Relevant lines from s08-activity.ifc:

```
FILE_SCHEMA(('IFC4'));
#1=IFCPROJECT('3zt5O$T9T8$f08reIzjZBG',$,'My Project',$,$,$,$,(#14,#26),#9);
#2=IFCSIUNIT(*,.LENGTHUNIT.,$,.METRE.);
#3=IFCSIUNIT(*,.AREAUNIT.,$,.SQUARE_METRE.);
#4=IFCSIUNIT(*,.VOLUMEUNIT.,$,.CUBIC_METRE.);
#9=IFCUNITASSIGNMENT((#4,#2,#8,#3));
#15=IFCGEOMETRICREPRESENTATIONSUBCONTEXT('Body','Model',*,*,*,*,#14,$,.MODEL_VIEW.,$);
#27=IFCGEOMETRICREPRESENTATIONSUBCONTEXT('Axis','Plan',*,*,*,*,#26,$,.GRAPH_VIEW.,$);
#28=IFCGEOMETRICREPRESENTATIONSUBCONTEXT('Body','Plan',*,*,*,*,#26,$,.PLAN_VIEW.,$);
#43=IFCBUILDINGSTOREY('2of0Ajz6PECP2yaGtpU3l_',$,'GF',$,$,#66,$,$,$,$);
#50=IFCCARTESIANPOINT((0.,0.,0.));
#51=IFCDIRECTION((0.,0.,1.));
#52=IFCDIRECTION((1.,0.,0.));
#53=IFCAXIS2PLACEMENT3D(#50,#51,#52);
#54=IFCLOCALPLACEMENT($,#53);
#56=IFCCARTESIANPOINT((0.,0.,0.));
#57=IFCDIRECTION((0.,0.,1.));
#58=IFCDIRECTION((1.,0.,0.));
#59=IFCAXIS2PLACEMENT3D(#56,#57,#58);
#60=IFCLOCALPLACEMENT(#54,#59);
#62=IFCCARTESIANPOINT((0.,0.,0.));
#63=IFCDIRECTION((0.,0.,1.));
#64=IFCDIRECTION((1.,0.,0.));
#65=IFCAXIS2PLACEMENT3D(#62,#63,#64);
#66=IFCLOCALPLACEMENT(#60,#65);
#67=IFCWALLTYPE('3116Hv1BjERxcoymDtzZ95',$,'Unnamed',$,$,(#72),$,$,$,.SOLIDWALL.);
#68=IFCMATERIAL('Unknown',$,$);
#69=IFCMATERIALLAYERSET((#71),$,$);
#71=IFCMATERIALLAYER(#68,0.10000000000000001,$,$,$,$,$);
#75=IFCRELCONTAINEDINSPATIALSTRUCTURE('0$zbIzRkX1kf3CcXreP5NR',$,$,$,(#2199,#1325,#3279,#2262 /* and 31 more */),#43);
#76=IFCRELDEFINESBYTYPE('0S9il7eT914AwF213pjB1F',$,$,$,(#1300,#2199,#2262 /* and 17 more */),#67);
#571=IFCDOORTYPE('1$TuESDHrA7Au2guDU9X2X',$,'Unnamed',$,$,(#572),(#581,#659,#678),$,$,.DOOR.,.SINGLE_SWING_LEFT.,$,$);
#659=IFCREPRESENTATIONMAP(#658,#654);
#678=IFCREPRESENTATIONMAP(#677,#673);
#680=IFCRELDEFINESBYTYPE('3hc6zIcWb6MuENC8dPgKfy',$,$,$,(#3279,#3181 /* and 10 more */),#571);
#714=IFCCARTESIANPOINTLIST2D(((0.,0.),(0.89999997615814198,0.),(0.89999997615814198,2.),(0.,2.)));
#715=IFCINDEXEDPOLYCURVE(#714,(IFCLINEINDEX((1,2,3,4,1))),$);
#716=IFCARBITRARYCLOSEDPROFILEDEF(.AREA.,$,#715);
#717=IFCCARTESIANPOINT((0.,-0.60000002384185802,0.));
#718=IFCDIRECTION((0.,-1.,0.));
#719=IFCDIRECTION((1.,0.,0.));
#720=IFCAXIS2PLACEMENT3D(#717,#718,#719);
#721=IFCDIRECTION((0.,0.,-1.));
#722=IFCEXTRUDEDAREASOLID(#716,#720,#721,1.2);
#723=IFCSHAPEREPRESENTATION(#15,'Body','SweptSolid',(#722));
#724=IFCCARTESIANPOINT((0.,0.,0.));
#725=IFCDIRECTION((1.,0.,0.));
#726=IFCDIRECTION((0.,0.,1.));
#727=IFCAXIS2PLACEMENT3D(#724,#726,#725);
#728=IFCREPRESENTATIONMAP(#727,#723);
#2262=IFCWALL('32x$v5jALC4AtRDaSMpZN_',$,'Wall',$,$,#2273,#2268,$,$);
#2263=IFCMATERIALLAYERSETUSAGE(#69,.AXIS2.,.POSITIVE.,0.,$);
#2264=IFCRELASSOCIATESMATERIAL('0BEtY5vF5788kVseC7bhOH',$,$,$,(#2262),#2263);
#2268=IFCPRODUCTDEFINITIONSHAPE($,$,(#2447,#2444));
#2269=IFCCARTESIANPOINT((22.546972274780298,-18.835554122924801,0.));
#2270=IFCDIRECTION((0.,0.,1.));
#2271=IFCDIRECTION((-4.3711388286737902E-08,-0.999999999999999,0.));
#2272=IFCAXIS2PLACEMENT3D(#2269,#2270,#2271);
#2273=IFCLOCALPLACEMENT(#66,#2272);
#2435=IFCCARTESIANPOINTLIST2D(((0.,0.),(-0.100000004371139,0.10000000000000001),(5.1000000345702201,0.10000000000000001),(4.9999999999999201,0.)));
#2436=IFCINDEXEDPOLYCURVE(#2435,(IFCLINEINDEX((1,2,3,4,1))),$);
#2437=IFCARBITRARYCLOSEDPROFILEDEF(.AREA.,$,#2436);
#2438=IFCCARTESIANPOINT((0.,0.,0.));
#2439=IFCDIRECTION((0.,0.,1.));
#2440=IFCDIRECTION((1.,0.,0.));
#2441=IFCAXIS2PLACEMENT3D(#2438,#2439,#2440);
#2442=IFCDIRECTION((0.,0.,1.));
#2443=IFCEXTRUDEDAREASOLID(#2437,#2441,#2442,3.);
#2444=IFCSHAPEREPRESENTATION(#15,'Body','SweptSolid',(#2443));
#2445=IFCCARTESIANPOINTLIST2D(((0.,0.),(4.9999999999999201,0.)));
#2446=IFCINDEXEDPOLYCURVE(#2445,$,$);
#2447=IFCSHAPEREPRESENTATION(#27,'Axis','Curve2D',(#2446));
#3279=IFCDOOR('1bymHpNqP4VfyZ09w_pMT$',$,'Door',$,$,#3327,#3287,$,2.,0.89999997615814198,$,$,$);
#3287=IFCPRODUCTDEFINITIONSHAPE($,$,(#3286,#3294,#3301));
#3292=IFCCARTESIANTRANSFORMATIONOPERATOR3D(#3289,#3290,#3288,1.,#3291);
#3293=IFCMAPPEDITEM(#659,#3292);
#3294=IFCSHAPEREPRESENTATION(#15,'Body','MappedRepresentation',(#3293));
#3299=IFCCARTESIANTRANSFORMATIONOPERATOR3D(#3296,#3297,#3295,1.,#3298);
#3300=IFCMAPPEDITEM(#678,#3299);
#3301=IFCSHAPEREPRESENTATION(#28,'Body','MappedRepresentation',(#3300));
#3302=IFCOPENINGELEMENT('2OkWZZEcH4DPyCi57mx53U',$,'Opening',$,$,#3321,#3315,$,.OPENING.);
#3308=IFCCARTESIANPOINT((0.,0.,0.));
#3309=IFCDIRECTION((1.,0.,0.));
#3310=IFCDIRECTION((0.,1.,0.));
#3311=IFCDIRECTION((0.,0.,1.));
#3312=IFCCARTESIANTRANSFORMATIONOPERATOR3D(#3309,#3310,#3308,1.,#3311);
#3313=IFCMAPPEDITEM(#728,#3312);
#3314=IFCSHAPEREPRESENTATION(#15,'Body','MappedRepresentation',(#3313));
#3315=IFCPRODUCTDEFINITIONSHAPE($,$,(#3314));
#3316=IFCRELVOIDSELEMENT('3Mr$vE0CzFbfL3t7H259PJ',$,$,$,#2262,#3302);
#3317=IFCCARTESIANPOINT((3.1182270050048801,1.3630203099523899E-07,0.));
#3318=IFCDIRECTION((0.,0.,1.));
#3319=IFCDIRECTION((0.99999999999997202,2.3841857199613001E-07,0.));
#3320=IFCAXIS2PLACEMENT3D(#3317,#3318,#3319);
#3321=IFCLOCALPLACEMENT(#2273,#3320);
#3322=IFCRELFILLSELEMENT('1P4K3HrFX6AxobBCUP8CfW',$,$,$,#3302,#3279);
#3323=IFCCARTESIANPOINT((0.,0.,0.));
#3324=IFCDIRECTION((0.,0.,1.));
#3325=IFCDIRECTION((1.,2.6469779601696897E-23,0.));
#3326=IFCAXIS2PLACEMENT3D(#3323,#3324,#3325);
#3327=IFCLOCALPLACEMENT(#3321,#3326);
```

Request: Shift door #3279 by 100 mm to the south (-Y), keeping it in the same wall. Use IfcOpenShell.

```python
import ifcopenshell
import ifcopenshell.api.geometry
import ifcopenshell.util.placement

model = ifcopenshell.open("s08-activity.ifc")

door = model.by_id(3279)
opening = door.FillsVoids[0].RelatingOpeningElement
wall = opening.VoidsElements[0].RelatingBuildingElement

wall_matrix = ifcopenshell.util.placement.get_local_placement(wall.ObjectPlacement)
shift = wall_matrix[:3, 0] * 0.1
before = ifcopenshell.util.placement.get_local_placement(door.ObjectPlacement)[:3, 3].copy()

# The door is placed relative to its opening, so it follows when the opening moves.
matrix = ifcopenshell.util.placement.get_local_placement(opening.ObjectPlacement)
matrix[:3, 3] += shift
ifcopenshell.api.geometry.edit_object_placement(
    model, product=opening, matrix=matrix, is_si=False, should_transform_children=True
)

after = ifcopenshell.util.placement.get_local_placement(door.ObjectPlacement)[:3, 3]
print("door moved by", (after - before).round(3) + 0.0)

model.write("s08-activity_v2.ifc")
```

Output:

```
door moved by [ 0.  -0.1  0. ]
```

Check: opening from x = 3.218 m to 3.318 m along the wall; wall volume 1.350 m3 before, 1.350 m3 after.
